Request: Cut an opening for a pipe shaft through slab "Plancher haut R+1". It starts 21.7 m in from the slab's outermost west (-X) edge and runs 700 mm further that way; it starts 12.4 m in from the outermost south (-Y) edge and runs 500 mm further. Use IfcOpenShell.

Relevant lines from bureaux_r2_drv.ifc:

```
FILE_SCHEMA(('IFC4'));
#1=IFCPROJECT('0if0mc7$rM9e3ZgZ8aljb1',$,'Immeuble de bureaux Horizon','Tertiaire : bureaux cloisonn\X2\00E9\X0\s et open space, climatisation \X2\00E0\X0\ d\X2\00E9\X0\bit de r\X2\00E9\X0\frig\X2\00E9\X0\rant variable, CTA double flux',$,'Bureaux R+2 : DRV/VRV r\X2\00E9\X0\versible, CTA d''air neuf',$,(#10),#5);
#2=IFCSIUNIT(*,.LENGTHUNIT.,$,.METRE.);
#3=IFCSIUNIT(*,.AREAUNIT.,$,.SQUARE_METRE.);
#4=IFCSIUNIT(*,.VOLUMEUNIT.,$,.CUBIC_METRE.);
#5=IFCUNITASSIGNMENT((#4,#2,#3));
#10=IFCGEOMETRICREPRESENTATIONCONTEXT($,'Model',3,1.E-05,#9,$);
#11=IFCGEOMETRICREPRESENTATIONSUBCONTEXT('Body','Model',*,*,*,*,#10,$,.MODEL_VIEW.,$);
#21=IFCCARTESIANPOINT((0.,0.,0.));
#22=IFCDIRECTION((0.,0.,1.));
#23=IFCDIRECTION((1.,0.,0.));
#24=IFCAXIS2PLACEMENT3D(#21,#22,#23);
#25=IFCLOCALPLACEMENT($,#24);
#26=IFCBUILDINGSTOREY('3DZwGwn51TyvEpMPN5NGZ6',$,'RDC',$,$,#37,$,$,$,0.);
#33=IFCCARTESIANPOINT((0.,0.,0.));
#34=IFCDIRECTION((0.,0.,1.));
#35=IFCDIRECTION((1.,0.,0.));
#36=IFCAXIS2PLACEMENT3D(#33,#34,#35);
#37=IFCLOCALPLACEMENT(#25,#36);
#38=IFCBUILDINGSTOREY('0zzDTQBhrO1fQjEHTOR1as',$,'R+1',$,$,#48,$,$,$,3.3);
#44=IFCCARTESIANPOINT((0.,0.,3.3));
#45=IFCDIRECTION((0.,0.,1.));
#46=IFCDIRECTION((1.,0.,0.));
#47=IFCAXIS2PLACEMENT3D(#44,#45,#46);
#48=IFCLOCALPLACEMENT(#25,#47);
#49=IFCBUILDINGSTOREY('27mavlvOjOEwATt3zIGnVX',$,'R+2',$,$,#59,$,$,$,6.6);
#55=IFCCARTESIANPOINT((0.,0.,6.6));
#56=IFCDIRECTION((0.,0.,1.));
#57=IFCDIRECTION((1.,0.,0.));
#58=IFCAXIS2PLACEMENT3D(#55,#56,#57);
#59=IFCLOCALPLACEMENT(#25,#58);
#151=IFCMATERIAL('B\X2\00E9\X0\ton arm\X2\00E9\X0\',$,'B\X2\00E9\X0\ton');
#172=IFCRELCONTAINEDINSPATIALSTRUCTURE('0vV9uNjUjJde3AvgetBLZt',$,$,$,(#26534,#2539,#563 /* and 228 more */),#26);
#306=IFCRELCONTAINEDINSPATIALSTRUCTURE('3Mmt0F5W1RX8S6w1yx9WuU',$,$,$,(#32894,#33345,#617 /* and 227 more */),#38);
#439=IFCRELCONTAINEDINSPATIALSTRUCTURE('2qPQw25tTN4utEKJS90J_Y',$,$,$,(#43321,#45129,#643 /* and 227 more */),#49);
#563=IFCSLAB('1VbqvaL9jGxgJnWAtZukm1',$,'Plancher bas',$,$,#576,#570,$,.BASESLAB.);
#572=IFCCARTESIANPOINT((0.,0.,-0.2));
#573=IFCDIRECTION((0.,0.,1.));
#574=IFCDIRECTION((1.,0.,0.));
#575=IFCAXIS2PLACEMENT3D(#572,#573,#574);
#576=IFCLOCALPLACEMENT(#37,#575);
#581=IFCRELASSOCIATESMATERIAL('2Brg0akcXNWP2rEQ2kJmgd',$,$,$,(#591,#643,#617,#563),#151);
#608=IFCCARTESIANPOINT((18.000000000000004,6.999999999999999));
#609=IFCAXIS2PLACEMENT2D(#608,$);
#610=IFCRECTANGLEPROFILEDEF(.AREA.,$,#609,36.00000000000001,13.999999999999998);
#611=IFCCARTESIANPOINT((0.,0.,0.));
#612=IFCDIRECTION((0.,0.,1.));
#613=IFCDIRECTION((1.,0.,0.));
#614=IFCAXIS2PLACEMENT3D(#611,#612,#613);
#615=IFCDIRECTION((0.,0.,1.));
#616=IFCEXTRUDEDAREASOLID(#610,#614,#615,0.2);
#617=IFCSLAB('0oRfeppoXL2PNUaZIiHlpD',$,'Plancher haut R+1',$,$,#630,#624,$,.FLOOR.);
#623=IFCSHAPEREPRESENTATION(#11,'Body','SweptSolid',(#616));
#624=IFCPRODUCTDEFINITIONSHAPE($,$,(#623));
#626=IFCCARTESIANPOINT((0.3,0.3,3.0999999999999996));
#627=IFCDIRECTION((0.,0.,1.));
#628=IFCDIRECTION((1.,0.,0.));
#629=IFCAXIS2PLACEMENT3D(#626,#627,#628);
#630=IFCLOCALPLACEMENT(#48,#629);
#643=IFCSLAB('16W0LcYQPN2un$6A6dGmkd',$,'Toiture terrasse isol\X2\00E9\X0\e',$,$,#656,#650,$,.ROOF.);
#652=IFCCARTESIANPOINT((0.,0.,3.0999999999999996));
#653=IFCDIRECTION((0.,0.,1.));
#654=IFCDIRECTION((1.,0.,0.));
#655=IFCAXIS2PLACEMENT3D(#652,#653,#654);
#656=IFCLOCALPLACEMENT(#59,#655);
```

```python
import numpy as np
import ifcopenshell
import ifcopenshell.api.feature
import ifcopenshell.api.geometry
import ifcopenshell.api.root
import ifcopenshell.geom
import ifcopenshell.util.placement
import ifcopenshell.util.representation
import ifcopenshell.util.shape
import ifcopenshell.util.unit

model = ifcopenshell.open("bureaux_r2_drv.ifc")
unit_scale = ifcopenshell.util.unit.calculate_unit_scale(model)
settings = ifcopenshell.geom.settings()


def volume(element):
    """Net volume in cubic metres, openings subtracted."""
    shape = ifcopenshell.geom.create_shape(settings, element)
    return ifcopenshell.util.shape.get_volume(shape.geometry)


slab = model.by_guid("0oRfeppoXL2PNUaZIiHlpD")
before = volume(slab)

# Extent in the slab's own axes, in metres. The edges named are its -X and -Y sides.
slab_shape = ifcopenshell.geom.create_shape(settings, slab)
vertices = ifcopenshell.util.shape.get_vertices(slab_shape.geometry)
x_min, y_min, bottom = vertices.min(axis=0)
top = vertices[:, 2].max()

opening = ifcopenshell.api.root.create_entity(model, ifc_class="IfcOpeningElement", name="Pipe shaft opening", predefined_type="OPENING")
context = ifcopenshell.util.representation.get_context(model, "Model", "Body", "MODEL_VIEW")
width, depth = 0.7, 0.5
outline = [(0.0, 0.0), (width, 0.0), (width, depth), (0.0, depth), (0.0, 0.0)]
# Overshoot both faces by 50 mm so the cut is clean.
shape = ifcopenshell.api.geometry.add_slab_representation(
    model, context=context, depth=top - bottom + 0.1, polyline=outline
)
ifcopenshell.api.geometry.assign_representation(model, product=opening, representation=shape)

matrix = ifcopenshell.util.placement.get_local_placement(slab.ObjectPlacement)
matrix[:, 3] = matrix @ np.append(np.array([x_min + 21.7, y_min + 12.4, bottom - 0.05]) / unit_scale, 1.0)
ifcopenshell.api.geometry.edit_object_placement(model, product=opening, matrix=matrix, is_si=False)
ifcopenshell.api.feature.add_feature(model, feature=opening, element=slab)

after = volume(slab)

print(f"slab volume {before:.3f} -> {after:.3f} m3")

model.write("bureaux_r2_drv_updated.ifc")
```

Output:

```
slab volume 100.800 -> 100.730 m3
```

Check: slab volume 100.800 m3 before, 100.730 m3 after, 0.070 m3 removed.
